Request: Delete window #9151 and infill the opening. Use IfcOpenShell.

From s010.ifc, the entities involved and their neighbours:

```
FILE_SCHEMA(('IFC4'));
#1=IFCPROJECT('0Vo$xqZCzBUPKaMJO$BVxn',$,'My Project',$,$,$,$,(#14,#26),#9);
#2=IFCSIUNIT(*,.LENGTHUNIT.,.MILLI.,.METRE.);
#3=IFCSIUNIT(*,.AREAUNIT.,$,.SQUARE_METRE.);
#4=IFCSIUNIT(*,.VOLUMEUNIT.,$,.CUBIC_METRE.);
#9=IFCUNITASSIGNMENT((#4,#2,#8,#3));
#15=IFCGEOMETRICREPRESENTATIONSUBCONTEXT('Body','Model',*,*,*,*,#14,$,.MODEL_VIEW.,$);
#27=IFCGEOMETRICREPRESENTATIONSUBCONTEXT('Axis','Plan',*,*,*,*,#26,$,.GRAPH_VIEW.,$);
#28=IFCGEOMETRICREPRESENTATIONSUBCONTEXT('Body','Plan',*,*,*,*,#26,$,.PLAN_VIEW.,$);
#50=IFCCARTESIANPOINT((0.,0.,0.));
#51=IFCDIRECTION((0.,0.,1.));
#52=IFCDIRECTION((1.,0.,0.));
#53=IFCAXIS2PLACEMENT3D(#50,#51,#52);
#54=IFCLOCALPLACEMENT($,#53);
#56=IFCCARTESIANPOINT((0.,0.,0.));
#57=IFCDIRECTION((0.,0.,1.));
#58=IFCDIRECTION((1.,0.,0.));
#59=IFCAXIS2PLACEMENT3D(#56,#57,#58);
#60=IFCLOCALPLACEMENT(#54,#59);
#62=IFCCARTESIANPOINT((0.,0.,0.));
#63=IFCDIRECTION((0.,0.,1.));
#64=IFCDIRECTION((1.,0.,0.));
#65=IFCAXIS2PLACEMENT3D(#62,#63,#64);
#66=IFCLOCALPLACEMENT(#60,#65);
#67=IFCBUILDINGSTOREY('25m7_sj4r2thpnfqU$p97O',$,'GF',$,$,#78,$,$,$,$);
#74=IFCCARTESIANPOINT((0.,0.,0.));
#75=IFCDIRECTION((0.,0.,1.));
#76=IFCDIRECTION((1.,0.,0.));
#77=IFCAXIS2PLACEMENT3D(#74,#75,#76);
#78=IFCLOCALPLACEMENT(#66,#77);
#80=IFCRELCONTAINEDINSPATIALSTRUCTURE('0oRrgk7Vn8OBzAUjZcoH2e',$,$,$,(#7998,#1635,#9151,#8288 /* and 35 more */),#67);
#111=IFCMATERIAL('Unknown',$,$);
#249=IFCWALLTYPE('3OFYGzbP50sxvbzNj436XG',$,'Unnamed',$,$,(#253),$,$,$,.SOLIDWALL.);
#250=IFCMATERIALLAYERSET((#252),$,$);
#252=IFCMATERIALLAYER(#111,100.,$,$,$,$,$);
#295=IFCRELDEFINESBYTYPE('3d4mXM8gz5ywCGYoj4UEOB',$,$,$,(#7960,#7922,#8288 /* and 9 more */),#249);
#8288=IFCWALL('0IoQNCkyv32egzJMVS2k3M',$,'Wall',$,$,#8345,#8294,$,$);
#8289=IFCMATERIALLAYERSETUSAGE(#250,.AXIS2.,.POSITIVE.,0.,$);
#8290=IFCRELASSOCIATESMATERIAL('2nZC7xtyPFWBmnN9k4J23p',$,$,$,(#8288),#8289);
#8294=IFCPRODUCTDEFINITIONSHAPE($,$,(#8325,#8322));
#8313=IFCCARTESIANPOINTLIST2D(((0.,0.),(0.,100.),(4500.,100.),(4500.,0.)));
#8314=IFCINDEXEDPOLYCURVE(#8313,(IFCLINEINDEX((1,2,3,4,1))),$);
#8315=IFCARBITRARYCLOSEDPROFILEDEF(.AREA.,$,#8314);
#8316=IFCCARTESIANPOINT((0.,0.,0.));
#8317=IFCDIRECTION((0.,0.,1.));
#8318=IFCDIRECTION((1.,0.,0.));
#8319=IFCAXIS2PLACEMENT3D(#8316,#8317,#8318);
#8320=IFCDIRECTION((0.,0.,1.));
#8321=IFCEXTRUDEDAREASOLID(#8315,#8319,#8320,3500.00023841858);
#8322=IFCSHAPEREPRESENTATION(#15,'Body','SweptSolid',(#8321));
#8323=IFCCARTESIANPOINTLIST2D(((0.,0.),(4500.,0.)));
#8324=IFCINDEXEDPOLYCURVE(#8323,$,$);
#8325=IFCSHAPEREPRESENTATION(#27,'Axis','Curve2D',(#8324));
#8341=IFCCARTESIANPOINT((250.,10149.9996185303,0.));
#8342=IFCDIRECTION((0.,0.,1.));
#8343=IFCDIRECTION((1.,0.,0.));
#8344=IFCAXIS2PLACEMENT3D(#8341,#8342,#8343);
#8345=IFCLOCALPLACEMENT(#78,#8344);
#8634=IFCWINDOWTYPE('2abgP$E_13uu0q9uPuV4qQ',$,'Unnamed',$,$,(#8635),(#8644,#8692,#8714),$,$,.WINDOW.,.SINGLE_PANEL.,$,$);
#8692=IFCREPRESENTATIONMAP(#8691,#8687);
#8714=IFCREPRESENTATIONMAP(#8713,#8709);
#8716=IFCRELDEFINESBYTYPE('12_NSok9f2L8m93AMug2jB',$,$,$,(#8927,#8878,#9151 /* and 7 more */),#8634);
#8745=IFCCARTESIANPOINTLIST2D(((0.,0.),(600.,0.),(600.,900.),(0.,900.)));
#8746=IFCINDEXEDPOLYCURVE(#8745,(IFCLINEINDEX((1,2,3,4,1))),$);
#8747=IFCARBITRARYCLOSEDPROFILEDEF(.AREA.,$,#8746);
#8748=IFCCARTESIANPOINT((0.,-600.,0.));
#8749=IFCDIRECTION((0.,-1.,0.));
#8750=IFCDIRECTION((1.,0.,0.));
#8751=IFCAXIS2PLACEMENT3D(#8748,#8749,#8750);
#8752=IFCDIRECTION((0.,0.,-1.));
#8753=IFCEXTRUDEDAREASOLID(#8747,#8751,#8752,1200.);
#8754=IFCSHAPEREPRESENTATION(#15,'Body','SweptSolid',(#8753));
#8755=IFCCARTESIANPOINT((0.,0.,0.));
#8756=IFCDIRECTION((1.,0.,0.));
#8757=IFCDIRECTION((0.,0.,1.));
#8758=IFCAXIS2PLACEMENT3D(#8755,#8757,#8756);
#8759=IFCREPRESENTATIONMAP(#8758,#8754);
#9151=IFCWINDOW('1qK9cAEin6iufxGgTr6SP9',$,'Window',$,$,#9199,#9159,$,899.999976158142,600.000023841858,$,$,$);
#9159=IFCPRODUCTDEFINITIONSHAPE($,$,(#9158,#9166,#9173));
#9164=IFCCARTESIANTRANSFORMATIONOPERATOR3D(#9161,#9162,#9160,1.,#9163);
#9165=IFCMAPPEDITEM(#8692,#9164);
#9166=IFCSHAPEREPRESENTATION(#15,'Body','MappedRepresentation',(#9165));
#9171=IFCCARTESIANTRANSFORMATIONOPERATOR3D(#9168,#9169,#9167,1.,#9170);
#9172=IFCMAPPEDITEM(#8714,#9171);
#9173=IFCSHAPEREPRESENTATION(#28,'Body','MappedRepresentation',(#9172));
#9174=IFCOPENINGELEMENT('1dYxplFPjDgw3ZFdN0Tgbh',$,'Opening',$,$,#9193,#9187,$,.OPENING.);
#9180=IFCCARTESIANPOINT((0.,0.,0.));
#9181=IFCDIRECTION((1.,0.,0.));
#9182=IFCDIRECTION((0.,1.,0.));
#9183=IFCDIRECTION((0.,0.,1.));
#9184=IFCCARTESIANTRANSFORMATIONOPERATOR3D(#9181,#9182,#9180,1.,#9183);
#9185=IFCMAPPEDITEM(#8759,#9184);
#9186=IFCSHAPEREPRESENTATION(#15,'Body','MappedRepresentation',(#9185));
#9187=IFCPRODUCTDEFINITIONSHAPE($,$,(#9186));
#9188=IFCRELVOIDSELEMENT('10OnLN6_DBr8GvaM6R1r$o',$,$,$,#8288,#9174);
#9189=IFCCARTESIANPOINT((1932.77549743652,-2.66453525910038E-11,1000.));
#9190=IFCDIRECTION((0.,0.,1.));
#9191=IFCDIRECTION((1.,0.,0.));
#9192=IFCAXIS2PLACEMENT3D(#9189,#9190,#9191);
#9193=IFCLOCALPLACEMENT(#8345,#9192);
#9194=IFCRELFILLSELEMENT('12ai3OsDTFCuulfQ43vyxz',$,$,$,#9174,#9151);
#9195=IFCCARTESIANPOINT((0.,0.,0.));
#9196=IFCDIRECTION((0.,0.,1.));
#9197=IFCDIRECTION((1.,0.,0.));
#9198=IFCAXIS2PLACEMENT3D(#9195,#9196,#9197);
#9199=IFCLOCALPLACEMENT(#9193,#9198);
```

```python
import ifcopenshell
import ifcopenshell.api.feature
import ifcopenshell.api.root
import ifcopenshell.geom
import ifcopenshell.util.shape

model = ifcopenshell.open("s010.ifc")
settings = ifcopenshell.geom.settings()


def volume(element):
    """Net volume in cubic metres, openings subtracted."""
    shape = ifcopenshell.geom.create_shape(settings, element)
    return ifcopenshell.util.shape.get_volume(shape.geometry)


window = model.by_guid("1qK9cAEin6iufxGgTr6SP9")
opening = window.FillsVoids[0].RelatingOpeningElement
wall = opening.VoidsElements[0].RelatingBuildingElement
before = volume(wall)

ifcopenshell.api.root.remove_product(model, product=window)
ifcopenshell.api.feature.remove_feature(model, feature=opening)

after = volume(wall)

print(f"wall volume {before:.3f} -> {after:.3f} m3")

model.write("s010-out.ifc")
```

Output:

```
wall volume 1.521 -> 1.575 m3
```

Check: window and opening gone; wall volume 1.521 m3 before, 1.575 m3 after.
